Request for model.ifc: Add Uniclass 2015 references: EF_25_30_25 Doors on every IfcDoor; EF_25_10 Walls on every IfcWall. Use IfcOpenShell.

First a look at what the model holds.

```python
import ifcopenshell

model = ifcopenshell.open("model.ifc")
print(model.schema)
print("classifications:", [c.Name for c in model.by_type("IfcClassification")])
for ifc_class in ("IfcDoor", "IfcRoof", "IfcStair", "IfcWall", "IfcWindow"):
    print(ifc_class, len(model.by_type(ifc_class)))
```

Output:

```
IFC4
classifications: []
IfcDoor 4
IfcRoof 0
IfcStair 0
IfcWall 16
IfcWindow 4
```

```python
import ifcopenshell
import ifcopenshell.api.classification

model = ifcopenshell.open("model.ifc")

system = ifcopenshell.api.classification.add_classification(model, classification="Uniclass 2015")

codes = {
    "IfcDoor": ("EF_25_30_25", "Doors"),
    "IfcWall": ("EF_25_10", "Walls"),
}
for ifc_class, (code, name) in codes.items():
    products = model.by_type(ifc_class)
    ifcopenshell.api.classification.add_reference(
        model, products=products, classification=system, identification=code, name=name
    )
    print(code, len(products))

model.write("model_v2.ifc")
```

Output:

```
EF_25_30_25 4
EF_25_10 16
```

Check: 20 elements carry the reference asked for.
